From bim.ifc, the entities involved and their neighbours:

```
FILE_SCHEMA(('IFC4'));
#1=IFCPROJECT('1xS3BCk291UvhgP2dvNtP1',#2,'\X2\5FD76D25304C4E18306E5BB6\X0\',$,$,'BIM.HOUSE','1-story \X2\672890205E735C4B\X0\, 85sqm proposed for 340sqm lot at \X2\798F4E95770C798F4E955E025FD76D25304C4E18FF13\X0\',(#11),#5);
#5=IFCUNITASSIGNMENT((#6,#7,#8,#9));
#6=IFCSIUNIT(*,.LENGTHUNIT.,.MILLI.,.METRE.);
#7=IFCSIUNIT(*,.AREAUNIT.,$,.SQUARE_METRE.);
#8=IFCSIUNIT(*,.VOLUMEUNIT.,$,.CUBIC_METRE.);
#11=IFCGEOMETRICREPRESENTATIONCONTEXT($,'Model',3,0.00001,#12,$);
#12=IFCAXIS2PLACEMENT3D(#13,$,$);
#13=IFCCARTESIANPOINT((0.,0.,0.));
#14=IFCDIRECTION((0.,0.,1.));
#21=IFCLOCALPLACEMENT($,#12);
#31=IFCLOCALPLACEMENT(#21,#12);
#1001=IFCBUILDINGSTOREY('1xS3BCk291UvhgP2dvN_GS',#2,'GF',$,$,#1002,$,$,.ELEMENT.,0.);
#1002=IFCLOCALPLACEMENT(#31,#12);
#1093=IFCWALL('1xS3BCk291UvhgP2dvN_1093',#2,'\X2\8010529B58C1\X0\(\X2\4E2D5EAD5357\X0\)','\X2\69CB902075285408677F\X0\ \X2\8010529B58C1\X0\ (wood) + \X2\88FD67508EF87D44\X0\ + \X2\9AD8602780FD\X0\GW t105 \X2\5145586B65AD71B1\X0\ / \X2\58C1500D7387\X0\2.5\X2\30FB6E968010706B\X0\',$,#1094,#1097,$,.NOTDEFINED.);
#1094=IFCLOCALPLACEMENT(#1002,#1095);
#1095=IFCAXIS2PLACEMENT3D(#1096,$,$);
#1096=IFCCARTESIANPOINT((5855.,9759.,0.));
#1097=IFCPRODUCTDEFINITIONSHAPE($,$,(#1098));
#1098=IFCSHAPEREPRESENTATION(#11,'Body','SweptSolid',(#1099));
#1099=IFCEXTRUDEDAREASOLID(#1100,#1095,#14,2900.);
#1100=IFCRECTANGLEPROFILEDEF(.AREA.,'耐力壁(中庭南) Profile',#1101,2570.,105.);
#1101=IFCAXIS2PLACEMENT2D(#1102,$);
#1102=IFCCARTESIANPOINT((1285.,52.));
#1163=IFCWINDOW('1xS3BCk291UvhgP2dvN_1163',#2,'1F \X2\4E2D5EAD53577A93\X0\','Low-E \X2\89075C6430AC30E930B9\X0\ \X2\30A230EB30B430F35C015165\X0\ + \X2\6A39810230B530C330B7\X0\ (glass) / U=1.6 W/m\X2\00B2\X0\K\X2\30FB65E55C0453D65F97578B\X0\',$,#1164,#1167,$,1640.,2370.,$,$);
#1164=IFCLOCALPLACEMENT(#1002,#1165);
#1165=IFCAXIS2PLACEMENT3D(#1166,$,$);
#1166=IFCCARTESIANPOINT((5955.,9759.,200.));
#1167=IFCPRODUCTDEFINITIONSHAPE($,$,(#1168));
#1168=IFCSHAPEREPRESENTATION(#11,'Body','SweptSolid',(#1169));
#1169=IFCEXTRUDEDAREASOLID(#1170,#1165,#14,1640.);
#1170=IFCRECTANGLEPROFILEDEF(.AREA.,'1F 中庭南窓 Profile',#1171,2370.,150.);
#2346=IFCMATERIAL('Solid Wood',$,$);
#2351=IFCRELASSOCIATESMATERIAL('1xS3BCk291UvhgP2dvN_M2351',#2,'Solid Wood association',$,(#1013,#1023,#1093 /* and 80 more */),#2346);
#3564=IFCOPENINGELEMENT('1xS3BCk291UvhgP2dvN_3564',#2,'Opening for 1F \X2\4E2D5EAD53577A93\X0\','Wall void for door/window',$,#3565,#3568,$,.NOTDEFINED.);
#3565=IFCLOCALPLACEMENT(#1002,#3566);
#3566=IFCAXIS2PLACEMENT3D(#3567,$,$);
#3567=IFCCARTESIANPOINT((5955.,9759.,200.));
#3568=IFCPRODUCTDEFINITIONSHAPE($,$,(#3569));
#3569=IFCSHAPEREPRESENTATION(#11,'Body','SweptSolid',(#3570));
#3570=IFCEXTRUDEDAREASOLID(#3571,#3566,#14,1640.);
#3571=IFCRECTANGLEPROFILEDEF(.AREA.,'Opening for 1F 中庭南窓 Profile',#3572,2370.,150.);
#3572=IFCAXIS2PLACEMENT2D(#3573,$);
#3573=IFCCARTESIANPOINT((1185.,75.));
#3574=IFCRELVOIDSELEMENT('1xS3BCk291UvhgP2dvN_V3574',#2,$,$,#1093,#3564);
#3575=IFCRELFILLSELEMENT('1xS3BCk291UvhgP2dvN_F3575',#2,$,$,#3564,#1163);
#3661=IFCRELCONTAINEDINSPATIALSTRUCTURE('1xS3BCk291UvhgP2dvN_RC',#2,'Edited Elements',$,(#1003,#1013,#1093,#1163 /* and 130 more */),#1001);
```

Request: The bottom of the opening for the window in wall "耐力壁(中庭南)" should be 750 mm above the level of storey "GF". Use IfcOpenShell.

```python
import numpy as np
import ifcopenshell
import ifcopenshell.api.geometry
import ifcopenshell.geom
import ifcopenshell.util.element
import ifcopenshell.util.placement
import ifcopenshell.util.shape
import ifcopenshell.util.unit

model = ifcopenshell.open("bim.ifc")
unit_scale = ifcopenshell.util.unit.calculate_unit_scale(model)

window = model.by_guid("1xS3BCk291UvhgP2dvN_1163")
opening = window.FillsVoids[0].RelatingOpeningElement
storey = ifcopenshell.util.element.get_container(window, ifc_class="IfcBuildingStorey")
level = ifcopenshell.util.placement.get_local_placement(storey.ObjectPlacement)[2, 3]

# The opening's origin need not be at the sill, so measure its lowest point.
shape = ifcopenshell.geom.create_shape(ifcopenshell.geom.settings(), opening)
bottom = ifcopenshell.util.shape.get_shape_bottom_elevation(shape, shape.geometry) / unit_scale
dz = level + 0.75 / unit_scale - bottom

shift = np.array([0.0, 0.0, dz])
# The window is not placed relative to its opening, so move both.
for product in (opening, window):
    matrix = ifcopenshell.util.placement.get_local_placement(product.ObjectPlacement)
    matrix[:3, 3] += shift
    ifcopenshell.api.geometry.edit_object_placement(model, product=product, matrix=matrix, is_si=False)

print(f"moved by {dz * unit_scale:+.3f} m")

model.write("bim_updated.ifc")
```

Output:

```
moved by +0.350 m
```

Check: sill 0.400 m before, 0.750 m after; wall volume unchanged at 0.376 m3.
